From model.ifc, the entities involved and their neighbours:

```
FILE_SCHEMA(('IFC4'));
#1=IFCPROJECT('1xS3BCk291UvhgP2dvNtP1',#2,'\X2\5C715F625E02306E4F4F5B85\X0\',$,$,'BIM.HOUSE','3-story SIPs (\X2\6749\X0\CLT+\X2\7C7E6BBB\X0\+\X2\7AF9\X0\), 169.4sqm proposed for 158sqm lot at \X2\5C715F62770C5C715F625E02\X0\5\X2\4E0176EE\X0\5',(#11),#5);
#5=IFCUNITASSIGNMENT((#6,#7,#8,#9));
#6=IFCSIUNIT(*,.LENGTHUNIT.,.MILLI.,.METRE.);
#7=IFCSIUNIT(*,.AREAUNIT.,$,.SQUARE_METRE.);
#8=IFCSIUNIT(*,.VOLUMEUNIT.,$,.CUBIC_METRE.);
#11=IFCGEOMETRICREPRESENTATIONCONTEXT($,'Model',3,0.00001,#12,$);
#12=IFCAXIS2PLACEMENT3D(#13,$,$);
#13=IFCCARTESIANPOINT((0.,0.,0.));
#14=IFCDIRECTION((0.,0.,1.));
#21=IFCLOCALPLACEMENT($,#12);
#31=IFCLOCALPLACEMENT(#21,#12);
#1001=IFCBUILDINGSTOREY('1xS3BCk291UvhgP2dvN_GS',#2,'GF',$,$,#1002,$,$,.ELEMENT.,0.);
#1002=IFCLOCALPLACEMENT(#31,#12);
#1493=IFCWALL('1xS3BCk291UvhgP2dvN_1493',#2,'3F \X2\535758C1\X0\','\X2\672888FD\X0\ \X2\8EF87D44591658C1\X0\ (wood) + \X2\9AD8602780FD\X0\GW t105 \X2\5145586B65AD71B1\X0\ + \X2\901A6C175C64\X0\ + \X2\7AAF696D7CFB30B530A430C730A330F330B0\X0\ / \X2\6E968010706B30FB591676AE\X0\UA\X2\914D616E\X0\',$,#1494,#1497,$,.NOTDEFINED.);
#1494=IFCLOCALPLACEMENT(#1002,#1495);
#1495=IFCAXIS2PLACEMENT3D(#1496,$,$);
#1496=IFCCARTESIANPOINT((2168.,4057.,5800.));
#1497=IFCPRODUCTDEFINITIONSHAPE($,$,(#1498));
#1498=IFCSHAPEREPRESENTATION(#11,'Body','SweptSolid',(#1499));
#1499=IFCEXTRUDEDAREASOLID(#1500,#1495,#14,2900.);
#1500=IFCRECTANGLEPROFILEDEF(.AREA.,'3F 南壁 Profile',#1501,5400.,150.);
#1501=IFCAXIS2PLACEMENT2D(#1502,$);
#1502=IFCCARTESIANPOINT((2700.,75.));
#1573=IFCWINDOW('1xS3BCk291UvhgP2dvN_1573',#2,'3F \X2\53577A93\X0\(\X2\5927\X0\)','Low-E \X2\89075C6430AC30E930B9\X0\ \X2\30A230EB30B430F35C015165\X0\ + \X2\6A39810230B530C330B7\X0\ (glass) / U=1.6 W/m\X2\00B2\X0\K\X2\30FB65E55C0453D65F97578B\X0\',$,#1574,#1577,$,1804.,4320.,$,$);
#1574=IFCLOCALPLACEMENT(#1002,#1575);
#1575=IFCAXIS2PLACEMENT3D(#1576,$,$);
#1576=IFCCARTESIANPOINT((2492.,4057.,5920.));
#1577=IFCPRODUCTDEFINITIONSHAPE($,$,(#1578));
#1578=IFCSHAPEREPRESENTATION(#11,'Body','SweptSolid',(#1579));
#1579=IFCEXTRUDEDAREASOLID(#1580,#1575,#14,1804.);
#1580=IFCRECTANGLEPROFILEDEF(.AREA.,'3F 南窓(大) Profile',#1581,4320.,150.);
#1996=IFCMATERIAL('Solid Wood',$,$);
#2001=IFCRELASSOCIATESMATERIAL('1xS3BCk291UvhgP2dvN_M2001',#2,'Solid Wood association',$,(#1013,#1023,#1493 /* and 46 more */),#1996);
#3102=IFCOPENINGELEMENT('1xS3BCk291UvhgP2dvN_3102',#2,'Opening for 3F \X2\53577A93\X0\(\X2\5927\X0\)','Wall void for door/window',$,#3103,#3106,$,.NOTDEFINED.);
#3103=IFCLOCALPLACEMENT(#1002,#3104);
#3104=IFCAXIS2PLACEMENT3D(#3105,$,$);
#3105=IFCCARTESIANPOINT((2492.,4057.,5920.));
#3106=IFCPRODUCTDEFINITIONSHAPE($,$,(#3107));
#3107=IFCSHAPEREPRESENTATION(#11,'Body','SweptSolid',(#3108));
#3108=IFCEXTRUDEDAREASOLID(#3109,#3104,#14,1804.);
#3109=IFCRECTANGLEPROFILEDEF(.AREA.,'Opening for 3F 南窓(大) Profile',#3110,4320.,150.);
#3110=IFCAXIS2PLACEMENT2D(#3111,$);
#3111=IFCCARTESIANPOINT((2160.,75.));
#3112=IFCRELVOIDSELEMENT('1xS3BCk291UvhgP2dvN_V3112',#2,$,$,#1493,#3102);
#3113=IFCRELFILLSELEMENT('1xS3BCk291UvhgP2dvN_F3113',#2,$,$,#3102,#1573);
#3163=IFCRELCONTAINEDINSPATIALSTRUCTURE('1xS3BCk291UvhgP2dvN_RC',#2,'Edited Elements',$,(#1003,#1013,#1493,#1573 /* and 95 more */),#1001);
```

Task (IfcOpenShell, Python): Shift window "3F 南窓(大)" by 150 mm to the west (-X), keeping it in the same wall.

```python
import ifcopenshell
import ifcopenshell.api.geometry
import ifcopenshell.util.placement
import ifcopenshell.util.unit

model = ifcopenshell.open("model.ifc")
unit_scale = ifcopenshell.util.unit.calculate_unit_scale(model)

window = model.by_guid("1xS3BCk291UvhgP2dvN_1573")
opening = window.FillsVoids[0].RelatingOpeningElement
wall = opening.VoidsElements[0].RelatingBuildingElement

wall_matrix = ifcopenshell.util.placement.get_local_placement(wall.ObjectPlacement)
shift = wall_matrix[:3, 0] * -0.15 / unit_scale
before = ifcopenshell.util.placement.get_local_placement(window.ObjectPlacement)[:3, 3].copy()

# The window is not placed relative to its opening, so move both.
for product in (opening, window):
    matrix = ifcopenshell.util.placement.get_local_placement(product.ObjectPlacement)
    matrix[:3, 3] += shift
    ifcopenshell.api.geometry.edit_object_placement(model, product=product, matrix=matrix, is_si=False)

after = ifcopenshell.util.placement.get_local_placement(window.ObjectPlacement)[:3, 3]
print("window moved by", (after - before).round(3) + 0.0)

model.write("model_edited.ifc")
```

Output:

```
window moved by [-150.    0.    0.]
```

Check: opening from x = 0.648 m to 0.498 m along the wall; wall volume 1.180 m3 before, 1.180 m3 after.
